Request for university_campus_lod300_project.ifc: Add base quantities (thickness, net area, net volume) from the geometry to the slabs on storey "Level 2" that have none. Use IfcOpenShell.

First a look at what the model holds.

```python
import ifcopenshell
import ifcopenshell.util.element
import ifcopenshell.util.unit

model = ifcopenshell.open("university_campus_lod300_project.ifc")
print(model.schema)
for unit_type in ("LENGTHUNIT", "AREAUNIT", "VOLUMEUNIT"):
    print(unit_type, ifcopenshell.util.unit.calculate_unit_scale(model, unit_type))
storey = next(s for s in model.by_type("IfcBuildingStorey") if s.Name == "Level 2")
slabs = [e for e in ifcopenshell.util.element.get_decomposition(storey) if e.is_a("IfcSlab")]
for e in sorted(slabs, key=lambda e: e.id()):
    print(e.id(), e.is_a(), e.Name, list(ifcopenshell.util.element.get_psets(e, qtos_only=True)), sep=" | ")
```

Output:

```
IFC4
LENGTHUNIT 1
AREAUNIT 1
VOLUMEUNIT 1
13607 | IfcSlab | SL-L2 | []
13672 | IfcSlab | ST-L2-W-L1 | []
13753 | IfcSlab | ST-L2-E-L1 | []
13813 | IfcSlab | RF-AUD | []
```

```python
import ifcopenshell
import ifcopenshell.api.pset
import ifcopenshell.geom
import ifcopenshell.util.element
import ifcopenshell.util.shape
import ifcopenshell.util.unit

model = ifcopenshell.open("university_campus_lod300_project.ifc")
unit_scale = ifcopenshell.util.unit.calculate_unit_scale(model)
area_scale = ifcopenshell.util.unit.calculate_unit_scale(model, "AREAUNIT")
volume_scale = ifcopenshell.util.unit.calculate_unit_scale(model, "VOLUMEUNIT")
settings = ifcopenshell.geom.settings()

storey = next(s for s in model.by_type("IfcBuildingStorey") if s.Name == "Level 2")
slabs = [e for e in ifcopenshell.util.element.get_decomposition(storey) if e.is_a("IfcSlab")]

for e in sorted(slabs, key=lambda e: e.id()):
    if ifcopenshell.util.element.get_psets(e, qtos_only=True, should_inherit=False):
        continue
    # Geometry comes back in metres, in the element's own axes.
    shape = ifcopenshell.geom.create_shape(settings, e)
    values = {
        "Width": ifcopenshell.util.shape.get_z(shape.geometry) / unit_scale,
        "NetArea": ifcopenshell.util.shape.get_footprint_area(shape.geometry) / area_scale,
        "NetVolume": ifcopenshell.util.shape.get_volume(shape.geometry) / volume_scale,
    }
    qto = ifcopenshell.api.pset.add_qto(model, product=e, name="Qto_SlabBaseQuantities")
    ifcopenshell.api.pset.edit_qto(model, qto=qto, properties=values)
    print(e.id(), {k: round(v, 3) for k, v in values.items()})

model.write("university_campus_lod300_project-out.ifc")
```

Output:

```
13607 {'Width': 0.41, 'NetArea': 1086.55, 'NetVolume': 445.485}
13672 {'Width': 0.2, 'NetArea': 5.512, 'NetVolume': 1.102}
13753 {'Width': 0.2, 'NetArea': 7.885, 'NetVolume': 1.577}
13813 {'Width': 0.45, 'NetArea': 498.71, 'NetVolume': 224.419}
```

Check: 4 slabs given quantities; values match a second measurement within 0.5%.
